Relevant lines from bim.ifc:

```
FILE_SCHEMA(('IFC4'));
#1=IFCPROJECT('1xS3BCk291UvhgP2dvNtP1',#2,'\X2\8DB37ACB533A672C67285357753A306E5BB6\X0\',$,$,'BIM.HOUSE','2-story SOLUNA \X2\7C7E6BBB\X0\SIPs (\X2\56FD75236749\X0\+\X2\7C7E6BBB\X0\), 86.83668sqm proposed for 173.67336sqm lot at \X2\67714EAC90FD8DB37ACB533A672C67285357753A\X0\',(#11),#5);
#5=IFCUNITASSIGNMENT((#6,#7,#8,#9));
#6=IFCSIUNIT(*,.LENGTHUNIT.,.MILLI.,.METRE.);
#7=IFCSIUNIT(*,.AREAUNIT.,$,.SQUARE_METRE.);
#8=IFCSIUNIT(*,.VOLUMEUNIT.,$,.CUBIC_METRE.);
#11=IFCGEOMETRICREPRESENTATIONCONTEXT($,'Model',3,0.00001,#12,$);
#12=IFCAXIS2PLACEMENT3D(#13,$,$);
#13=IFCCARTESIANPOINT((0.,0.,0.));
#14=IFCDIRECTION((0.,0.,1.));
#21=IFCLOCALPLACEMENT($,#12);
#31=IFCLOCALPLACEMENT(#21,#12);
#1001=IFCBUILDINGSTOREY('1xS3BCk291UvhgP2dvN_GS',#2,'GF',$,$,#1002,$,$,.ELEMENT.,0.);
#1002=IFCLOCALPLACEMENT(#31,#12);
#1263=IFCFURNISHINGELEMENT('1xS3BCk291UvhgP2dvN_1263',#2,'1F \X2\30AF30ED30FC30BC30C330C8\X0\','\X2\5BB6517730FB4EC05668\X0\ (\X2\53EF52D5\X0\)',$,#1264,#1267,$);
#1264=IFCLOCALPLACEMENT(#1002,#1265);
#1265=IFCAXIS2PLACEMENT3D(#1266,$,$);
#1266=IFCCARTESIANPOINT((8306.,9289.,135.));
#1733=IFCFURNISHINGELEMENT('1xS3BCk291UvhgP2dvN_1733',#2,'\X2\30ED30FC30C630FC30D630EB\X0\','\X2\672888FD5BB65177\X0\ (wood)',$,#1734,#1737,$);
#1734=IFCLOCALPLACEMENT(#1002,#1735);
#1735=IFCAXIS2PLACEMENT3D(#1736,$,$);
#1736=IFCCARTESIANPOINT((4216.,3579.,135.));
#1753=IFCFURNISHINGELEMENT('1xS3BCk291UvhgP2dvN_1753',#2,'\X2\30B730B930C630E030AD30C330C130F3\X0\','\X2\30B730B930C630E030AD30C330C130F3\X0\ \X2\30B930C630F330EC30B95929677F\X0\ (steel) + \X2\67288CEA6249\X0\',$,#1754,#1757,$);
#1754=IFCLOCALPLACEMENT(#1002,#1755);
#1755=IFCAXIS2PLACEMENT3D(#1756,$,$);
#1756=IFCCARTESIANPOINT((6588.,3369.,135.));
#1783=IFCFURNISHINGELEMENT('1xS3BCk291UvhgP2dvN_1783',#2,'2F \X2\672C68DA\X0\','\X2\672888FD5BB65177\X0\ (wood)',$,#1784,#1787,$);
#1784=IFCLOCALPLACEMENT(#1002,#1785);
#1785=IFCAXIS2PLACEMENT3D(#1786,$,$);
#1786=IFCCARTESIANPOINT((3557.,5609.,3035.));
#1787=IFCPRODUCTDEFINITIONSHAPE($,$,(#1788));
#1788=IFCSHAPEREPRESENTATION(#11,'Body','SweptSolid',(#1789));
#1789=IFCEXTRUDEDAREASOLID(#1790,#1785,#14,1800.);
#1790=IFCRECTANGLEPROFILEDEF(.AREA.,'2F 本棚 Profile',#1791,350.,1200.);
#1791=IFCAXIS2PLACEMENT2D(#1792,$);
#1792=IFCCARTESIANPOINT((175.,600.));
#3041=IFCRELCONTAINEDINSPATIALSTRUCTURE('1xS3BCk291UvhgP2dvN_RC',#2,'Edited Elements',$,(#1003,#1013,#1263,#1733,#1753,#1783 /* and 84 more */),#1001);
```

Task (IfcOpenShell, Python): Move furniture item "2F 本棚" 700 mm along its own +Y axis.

```python
import ifcopenshell
import ifcopenshell.api.geometry
import ifcopenshell.util.placement
import ifcopenshell.util.unit

model = ifcopenshell.open("bim.ifc")
unit_scale = ifcopenshell.util.unit.calculate_unit_scale(model)

item = model.by_id(1783)
matrix = ifcopenshell.util.placement.get_local_placement(item.ObjectPlacement)
matrix[:3, 3] += matrix[:3, 1] * 0.7 / unit_scale
ifcopenshell.api.geometry.edit_object_placement(model, product=item, matrix=matrix, is_si=False)

print(ifcopenshell.util.placement.get_local_placement(item.ObjectPlacement).round(3) + 0.0)

model.write("bim_updated.ifc")
```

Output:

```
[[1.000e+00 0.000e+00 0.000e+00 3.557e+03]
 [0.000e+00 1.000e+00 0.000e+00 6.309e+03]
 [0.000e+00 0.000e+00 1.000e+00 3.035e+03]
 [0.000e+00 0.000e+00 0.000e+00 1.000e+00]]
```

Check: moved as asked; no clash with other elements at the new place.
